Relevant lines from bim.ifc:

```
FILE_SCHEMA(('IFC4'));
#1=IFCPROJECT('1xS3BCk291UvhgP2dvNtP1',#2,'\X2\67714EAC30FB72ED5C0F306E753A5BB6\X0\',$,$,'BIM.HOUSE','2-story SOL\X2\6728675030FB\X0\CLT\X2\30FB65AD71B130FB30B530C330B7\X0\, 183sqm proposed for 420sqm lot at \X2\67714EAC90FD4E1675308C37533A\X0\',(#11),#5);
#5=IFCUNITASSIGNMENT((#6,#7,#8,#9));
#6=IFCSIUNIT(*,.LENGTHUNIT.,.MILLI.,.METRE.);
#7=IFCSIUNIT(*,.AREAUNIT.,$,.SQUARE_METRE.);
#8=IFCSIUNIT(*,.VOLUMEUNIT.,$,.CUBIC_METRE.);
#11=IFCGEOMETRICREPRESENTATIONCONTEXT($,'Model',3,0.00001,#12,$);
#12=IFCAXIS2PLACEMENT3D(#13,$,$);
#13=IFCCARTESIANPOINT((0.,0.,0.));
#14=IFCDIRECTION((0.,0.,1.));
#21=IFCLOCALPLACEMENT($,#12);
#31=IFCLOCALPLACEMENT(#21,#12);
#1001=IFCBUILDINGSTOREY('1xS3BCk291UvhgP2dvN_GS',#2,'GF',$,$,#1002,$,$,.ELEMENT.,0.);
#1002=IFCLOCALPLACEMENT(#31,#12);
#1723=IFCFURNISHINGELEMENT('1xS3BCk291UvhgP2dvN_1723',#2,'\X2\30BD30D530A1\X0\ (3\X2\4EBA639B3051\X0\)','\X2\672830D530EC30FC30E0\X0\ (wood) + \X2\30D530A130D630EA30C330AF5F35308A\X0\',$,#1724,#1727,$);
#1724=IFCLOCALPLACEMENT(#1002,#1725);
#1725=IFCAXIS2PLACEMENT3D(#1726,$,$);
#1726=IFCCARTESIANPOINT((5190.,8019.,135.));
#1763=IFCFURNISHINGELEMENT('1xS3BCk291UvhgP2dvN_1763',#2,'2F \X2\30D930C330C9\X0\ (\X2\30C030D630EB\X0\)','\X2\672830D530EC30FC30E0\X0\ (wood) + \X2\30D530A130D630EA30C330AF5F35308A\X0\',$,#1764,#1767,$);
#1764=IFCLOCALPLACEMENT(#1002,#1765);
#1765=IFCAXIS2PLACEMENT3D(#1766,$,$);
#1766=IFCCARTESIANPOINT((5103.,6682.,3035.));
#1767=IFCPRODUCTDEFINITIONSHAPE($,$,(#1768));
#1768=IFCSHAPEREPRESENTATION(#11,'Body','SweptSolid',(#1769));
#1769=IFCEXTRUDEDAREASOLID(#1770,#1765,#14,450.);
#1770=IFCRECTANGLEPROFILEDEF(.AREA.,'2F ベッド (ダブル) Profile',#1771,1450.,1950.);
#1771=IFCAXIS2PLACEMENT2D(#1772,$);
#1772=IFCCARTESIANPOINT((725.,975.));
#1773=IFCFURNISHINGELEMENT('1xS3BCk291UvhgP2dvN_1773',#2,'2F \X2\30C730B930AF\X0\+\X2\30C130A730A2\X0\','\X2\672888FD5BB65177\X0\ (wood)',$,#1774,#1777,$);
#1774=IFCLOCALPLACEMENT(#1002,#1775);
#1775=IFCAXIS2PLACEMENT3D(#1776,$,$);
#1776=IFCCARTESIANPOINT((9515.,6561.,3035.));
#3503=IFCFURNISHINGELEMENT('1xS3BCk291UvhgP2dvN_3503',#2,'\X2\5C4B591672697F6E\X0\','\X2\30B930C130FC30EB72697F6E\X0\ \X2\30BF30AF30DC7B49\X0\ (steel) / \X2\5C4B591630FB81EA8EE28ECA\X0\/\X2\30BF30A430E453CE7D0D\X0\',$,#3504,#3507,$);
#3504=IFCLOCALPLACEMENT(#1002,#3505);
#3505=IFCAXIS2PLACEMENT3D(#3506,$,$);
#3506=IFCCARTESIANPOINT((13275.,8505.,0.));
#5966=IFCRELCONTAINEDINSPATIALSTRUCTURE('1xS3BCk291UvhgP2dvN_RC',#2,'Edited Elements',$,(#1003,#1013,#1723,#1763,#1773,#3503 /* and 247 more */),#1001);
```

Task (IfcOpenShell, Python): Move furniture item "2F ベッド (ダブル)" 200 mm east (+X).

```python
import ifcopenshell
import ifcopenshell.api.geometry
import ifcopenshell.util.placement
import ifcopenshell.util.unit

model = ifcopenshell.open("bim.ifc")
unit_scale = ifcopenshell.util.unit.calculate_unit_scale(model)

item = model.by_guid("1xS3BCk291UvhgP2dvN_1763")
matrix = ifcopenshell.util.placement.get_local_placement(item.ObjectPlacement)
matrix[0, 3] += 0.2 / unit_scale
ifcopenshell.api.geometry.edit_object_placement(model, product=item, matrix=matrix, is_si=False)

print(ifcopenshell.util.placement.get_local_placement(item.ObjectPlacement).round(3) + 0.0)

model.write("bim_rev.ifc")
```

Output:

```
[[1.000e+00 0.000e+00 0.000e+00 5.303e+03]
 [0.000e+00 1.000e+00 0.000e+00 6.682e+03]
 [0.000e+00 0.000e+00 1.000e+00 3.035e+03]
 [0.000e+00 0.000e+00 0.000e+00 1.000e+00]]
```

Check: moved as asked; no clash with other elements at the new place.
